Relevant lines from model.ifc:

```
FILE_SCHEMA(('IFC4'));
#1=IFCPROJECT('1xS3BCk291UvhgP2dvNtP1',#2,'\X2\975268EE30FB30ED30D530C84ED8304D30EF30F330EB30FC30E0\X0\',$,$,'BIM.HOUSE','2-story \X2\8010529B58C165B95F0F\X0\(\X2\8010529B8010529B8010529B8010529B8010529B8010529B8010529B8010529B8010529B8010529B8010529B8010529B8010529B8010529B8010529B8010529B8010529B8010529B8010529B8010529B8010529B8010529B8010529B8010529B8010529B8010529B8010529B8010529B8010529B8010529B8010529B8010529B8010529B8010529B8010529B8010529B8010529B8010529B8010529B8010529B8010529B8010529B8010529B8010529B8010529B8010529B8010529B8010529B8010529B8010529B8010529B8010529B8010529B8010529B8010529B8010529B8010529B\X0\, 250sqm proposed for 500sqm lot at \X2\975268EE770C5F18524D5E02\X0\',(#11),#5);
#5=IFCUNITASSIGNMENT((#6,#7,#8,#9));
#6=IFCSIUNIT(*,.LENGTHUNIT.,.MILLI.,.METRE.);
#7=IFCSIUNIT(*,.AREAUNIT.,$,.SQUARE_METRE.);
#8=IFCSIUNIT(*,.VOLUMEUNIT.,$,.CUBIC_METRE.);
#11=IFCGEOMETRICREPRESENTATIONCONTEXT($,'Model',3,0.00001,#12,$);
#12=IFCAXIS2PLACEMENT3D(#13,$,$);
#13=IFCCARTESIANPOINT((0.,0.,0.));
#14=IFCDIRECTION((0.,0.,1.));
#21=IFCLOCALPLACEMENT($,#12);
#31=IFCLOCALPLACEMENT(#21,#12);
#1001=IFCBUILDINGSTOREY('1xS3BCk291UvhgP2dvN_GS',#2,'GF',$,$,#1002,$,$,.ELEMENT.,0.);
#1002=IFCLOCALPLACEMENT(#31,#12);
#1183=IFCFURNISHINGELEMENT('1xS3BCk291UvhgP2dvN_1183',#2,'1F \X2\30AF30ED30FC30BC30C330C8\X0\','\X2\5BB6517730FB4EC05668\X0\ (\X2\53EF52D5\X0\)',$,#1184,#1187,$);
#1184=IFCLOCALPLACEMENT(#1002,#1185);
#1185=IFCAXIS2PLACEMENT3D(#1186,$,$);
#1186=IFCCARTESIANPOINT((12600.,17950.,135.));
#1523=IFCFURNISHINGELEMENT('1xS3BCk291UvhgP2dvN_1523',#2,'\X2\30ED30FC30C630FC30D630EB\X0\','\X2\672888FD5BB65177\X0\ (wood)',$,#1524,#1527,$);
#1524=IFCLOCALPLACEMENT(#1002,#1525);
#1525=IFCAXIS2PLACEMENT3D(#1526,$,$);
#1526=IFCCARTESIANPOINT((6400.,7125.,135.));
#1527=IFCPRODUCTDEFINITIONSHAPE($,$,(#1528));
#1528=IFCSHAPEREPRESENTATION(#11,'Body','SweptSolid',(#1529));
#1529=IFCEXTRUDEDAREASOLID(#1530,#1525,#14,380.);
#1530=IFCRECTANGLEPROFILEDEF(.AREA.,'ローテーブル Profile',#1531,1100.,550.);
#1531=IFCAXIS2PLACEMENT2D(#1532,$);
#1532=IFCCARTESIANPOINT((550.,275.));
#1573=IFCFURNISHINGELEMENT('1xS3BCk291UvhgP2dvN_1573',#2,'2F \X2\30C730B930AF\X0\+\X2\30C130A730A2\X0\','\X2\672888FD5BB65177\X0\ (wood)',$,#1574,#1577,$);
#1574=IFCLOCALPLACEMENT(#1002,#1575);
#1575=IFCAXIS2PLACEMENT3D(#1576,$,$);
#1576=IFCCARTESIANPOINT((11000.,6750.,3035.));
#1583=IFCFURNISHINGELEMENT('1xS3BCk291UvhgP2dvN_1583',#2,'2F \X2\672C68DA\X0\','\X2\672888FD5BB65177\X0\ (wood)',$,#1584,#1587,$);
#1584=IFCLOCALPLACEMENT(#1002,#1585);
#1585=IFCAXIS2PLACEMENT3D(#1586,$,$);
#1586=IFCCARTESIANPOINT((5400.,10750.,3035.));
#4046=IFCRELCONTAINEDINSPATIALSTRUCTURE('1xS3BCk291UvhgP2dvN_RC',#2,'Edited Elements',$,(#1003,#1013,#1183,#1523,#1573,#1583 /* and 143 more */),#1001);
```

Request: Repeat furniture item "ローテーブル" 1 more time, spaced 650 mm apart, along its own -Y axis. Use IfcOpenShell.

```python
import ifcopenshell
import ifcopenshell.api.geometry
import ifcopenshell.api.root
import ifcopenshell.util.element
import ifcopenshell.util.placement

model = ifcopenshell.open("model.ifc")


def reuse_history(source, copy):
    """copy_class also copies each property set's owner history, people and application; keep the originals."""
    for rel in copy.IsDefinedBy:
        if rel.is_a("IfcRelDefinesByProperties") and (history := rel.RelatingPropertyDefinition.OwnerHistory):
            rel.RelatingPropertyDefinition.OwnerHistory = source.OwnerHistory
            ifcopenshell.util.element.remove_deep2(model, history)


source = model.by_guid("1xS3BCk291UvhgP2dvN_1523")
base = ifcopenshell.util.placement.get_local_placement(source.ObjectPlacement)
step = -base[:3, 1] * 650.0

for i in range(1, 2):
    copy = ifcopenshell.api.root.copy_class(model, product=source)
    copy.Representation = ifcopenshell.util.element.copy_deep(
        model, source.Representation, exclude=["IfcGeometricRepresentationContext", "IfcRepresentationMap"]
    )
    reuse_history(source, copy)
    matrix = base.copy()
    matrix[:3, 3] += i * step
    print("added at", matrix[:3, 3].round(3) + 0.0)
    ifcopenshell.api.geometry.edit_object_placement(model, product=copy, matrix=matrix, is_si=False)

model.write("model_v2.ifc")
```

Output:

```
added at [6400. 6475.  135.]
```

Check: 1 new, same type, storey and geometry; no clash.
